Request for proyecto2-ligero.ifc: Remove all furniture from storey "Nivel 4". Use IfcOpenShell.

First a look at what the model holds.

```python
import ifcopenshell
import ifcopenshell.util.element

model = ifcopenshell.open("proyecto2-ligero.ifc")
print(model.schema)
storey = next(s for s in model.by_type("IfcBuildingStorey") if s.Name == "Nivel 4")
furniture = [e for e in ifcopenshell.util.element.get_decomposition(storey) if e.is_a("IfcFurnishingElement")]
seen = {}
for e in furniture:
    element_type = ifcopenshell.util.element.get_type(e)
    name = element_type.Name if element_type not in (None, e) else None
    seen[name] = seen.get(name, 0) + 1
for name, count in sorted(seen.items(), key=str):
    print(count, "x", name)
```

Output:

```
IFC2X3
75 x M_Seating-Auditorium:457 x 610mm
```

```python
import ifcopenshell
import ifcopenshell.api.root
import ifcopenshell.util.element

model = ifcopenshell.open("proyecto2-ligero.ifc")

storey = next(s for s in model.by_type("IfcBuildingStorey") if s.Name == "Nivel 4")
furniture = [e for e in ifcopenshell.util.element.get_decomposition(storey) if e.is_a("IfcFurnishingElement")]

for e in furniture:
    ifcopenshell.api.root.remove_product(model, product=e)
print(len(furniture), "removed")

model.write("proyecto2-ligero-out.ifc")
```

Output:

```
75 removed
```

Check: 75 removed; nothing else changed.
